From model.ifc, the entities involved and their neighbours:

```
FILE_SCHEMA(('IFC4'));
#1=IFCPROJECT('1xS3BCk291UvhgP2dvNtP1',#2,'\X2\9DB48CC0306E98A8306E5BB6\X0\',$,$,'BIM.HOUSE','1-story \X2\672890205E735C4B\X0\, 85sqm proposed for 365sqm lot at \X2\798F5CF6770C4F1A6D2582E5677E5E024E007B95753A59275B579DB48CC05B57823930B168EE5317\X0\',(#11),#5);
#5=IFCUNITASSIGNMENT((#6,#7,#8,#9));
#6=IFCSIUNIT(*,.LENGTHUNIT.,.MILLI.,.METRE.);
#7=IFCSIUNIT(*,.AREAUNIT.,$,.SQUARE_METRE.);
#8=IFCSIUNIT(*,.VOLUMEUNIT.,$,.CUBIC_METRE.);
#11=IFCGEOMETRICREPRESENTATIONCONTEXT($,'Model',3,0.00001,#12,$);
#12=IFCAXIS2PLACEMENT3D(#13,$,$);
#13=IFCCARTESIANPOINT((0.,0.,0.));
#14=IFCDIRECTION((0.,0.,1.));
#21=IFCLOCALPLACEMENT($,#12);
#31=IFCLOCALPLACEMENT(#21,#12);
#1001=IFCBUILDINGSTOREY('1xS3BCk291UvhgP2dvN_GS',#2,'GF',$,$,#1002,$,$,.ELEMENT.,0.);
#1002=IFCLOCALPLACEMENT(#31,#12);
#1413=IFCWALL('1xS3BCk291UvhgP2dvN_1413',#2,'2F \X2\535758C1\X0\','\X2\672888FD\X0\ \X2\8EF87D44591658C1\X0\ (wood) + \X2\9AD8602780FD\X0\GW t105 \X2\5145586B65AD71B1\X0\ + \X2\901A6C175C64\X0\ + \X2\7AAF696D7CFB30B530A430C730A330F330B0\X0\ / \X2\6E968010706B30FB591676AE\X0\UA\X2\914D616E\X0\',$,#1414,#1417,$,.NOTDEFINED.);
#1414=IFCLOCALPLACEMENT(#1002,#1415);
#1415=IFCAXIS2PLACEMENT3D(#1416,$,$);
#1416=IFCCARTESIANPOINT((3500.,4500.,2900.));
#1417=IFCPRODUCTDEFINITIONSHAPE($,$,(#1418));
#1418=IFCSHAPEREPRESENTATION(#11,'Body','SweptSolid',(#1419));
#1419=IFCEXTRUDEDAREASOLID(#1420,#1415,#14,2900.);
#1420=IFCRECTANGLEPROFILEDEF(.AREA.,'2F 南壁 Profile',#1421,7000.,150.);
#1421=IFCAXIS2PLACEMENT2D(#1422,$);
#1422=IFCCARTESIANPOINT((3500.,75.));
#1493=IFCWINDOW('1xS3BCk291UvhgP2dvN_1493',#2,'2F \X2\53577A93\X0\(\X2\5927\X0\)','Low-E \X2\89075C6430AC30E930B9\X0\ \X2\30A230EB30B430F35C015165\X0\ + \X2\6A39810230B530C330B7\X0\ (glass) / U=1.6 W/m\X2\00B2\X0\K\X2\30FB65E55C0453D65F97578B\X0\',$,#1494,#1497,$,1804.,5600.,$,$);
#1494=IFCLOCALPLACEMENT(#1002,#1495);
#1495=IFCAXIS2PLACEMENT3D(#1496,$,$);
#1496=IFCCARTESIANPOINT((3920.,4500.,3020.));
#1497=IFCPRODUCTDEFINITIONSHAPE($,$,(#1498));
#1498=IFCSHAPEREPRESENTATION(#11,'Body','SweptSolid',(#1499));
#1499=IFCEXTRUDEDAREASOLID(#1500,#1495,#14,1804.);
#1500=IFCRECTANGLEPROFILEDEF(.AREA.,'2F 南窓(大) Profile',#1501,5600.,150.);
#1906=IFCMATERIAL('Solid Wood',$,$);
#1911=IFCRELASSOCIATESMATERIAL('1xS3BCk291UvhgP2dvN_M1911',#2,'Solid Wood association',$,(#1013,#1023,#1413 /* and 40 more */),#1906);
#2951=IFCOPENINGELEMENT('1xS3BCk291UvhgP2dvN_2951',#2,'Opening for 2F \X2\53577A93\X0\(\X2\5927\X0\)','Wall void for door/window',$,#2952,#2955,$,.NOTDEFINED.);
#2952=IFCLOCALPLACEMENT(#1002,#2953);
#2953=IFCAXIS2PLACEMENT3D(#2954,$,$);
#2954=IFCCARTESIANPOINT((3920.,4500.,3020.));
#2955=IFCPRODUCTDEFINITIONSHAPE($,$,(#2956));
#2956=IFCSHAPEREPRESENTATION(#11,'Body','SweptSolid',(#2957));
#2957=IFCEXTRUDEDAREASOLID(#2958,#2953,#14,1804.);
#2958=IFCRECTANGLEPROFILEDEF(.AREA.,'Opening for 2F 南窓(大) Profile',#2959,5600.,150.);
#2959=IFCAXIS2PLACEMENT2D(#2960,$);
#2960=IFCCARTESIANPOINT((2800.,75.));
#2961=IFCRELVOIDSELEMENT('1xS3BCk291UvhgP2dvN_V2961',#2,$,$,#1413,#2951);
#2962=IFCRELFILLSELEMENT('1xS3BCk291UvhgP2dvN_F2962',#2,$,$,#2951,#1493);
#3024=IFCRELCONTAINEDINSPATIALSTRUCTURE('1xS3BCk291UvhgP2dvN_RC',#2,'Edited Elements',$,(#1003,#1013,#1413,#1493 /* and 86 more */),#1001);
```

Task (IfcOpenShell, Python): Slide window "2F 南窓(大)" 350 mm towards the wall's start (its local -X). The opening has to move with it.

```python
import ifcopenshell
import ifcopenshell.api.geometry
import ifcopenshell.util.placement
import ifcopenshell.util.unit

model = ifcopenshell.open("model.ifc")
unit_scale = ifcopenshell.util.unit.calculate_unit_scale(model)

window = model.by_guid("1xS3BCk291UvhgP2dvN_1493")
opening = window.FillsVoids[0].RelatingOpeningElement
wall = opening.VoidsElements[0].RelatingBuildingElement

wall_matrix = ifcopenshell.util.placement.get_local_placement(wall.ObjectPlacement)
shift = wall_matrix[:3, 0] * -0.35 / unit_scale
before = ifcopenshell.util.placement.get_local_placement(window.ObjectPlacement)[:3, 3].copy()

# The window is not placed relative to its opening, so move both.
for product in (opening, window):
    matrix = ifcopenshell.util.placement.get_local_placement(product.ObjectPlacement)
    matrix[:3, 3] += shift
    ifcopenshell.api.geometry.edit_object_placement(model, product=product, matrix=matrix, is_si=False)

after = ifcopenshell.util.placement.get_local_placement(window.ObjectPlacement)[:3, 3]
print("window moved by", (after - before).round(3) + 0.0)

model.write("model_v2.ifc")
```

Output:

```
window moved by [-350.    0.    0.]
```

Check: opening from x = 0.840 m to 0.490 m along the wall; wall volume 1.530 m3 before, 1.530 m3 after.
